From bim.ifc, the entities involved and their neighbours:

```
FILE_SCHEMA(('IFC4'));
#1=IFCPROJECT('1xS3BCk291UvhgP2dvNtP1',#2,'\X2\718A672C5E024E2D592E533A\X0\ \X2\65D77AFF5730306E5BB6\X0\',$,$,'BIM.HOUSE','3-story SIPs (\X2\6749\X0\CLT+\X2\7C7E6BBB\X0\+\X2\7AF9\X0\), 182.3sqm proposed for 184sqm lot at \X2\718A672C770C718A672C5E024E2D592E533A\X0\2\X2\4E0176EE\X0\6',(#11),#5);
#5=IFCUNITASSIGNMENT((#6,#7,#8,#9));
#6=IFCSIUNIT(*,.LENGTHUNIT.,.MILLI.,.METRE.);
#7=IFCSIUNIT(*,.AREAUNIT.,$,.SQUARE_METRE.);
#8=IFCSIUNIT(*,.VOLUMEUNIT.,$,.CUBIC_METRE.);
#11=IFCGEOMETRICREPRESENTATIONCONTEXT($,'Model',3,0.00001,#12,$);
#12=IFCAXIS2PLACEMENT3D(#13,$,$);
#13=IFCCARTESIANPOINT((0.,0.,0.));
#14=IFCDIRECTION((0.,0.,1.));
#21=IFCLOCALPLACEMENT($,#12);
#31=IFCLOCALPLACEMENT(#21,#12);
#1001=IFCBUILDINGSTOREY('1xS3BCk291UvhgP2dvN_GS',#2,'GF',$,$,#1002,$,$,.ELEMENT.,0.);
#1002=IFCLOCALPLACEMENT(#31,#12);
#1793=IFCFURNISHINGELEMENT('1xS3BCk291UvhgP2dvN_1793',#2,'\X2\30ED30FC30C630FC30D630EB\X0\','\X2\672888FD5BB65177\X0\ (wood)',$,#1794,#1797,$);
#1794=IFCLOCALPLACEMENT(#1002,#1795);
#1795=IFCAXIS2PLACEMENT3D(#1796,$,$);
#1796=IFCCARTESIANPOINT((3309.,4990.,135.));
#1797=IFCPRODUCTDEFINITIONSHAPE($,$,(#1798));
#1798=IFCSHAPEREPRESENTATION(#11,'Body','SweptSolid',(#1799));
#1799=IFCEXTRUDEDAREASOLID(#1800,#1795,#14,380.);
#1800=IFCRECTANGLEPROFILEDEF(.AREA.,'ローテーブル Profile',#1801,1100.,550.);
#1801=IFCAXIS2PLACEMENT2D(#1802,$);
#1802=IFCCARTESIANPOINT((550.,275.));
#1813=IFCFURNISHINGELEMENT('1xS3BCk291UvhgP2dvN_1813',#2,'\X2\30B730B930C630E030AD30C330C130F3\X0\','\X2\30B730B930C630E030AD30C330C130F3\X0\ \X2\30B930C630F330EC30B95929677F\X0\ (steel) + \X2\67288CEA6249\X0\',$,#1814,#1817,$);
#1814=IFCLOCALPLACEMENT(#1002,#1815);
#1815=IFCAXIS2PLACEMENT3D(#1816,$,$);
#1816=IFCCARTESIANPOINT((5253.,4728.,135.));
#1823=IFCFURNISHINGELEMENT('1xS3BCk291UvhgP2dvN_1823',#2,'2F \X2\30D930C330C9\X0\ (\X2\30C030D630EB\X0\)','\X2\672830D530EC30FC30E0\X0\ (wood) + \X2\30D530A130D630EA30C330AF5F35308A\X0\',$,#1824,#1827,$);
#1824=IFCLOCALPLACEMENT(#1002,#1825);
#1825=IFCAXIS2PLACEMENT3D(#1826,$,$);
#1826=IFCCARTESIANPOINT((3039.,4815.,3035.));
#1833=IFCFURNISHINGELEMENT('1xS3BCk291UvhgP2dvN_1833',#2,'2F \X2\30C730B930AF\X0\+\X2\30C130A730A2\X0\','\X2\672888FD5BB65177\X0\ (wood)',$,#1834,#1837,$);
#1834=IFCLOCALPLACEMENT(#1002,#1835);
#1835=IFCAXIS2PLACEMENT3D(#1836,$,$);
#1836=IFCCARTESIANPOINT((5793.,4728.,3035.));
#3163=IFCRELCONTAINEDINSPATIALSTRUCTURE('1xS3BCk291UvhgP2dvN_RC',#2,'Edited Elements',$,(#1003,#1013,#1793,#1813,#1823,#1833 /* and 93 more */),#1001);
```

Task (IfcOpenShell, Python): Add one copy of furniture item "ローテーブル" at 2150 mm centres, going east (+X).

```python
import numpy as np
import ifcopenshell
import ifcopenshell.api.geometry
import ifcopenshell.api.root
import ifcopenshell.util.element
import ifcopenshell.util.placement

model = ifcopenshell.open("bim.ifc")


def reuse_history(source, copy):
    """copy_class also copies each property set's owner history, people and application; keep the originals."""
    for rel in copy.IsDefinedBy:
        if rel.is_a("IfcRelDefinesByProperties") and (history := rel.RelatingPropertyDefinition.OwnerHistory):
            rel.RelatingPropertyDefinition.OwnerHistory = source.OwnerHistory
            ifcopenshell.util.element.remove_deep2(model, history)


source = model.by_id(1793)
base = ifcopenshell.util.placement.get_local_placement(source.ObjectPlacement)
step = np.array([1.0, 0.0, 0.0]) * 2150.0

for i in range(1, 2):
    copy = ifcopenshell.api.root.copy_class(model, product=source)
    copy.Representation = ifcopenshell.util.element.copy_deep(
        model, source.Representation, exclude=["IfcGeometricRepresentationContext", "IfcRepresentationMap"]
    )
    reuse_history(source, copy)
    matrix = base.copy()
    matrix[:3, 3] += i * step
    print("added at", matrix[:3, 3].round(3) + 0.0)
    ifcopenshell.api.geometry.edit_object_placement(model, product=copy, matrix=matrix, is_si=False)

model.write("bim_v2.ifc")
```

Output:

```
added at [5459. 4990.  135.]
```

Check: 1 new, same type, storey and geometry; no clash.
